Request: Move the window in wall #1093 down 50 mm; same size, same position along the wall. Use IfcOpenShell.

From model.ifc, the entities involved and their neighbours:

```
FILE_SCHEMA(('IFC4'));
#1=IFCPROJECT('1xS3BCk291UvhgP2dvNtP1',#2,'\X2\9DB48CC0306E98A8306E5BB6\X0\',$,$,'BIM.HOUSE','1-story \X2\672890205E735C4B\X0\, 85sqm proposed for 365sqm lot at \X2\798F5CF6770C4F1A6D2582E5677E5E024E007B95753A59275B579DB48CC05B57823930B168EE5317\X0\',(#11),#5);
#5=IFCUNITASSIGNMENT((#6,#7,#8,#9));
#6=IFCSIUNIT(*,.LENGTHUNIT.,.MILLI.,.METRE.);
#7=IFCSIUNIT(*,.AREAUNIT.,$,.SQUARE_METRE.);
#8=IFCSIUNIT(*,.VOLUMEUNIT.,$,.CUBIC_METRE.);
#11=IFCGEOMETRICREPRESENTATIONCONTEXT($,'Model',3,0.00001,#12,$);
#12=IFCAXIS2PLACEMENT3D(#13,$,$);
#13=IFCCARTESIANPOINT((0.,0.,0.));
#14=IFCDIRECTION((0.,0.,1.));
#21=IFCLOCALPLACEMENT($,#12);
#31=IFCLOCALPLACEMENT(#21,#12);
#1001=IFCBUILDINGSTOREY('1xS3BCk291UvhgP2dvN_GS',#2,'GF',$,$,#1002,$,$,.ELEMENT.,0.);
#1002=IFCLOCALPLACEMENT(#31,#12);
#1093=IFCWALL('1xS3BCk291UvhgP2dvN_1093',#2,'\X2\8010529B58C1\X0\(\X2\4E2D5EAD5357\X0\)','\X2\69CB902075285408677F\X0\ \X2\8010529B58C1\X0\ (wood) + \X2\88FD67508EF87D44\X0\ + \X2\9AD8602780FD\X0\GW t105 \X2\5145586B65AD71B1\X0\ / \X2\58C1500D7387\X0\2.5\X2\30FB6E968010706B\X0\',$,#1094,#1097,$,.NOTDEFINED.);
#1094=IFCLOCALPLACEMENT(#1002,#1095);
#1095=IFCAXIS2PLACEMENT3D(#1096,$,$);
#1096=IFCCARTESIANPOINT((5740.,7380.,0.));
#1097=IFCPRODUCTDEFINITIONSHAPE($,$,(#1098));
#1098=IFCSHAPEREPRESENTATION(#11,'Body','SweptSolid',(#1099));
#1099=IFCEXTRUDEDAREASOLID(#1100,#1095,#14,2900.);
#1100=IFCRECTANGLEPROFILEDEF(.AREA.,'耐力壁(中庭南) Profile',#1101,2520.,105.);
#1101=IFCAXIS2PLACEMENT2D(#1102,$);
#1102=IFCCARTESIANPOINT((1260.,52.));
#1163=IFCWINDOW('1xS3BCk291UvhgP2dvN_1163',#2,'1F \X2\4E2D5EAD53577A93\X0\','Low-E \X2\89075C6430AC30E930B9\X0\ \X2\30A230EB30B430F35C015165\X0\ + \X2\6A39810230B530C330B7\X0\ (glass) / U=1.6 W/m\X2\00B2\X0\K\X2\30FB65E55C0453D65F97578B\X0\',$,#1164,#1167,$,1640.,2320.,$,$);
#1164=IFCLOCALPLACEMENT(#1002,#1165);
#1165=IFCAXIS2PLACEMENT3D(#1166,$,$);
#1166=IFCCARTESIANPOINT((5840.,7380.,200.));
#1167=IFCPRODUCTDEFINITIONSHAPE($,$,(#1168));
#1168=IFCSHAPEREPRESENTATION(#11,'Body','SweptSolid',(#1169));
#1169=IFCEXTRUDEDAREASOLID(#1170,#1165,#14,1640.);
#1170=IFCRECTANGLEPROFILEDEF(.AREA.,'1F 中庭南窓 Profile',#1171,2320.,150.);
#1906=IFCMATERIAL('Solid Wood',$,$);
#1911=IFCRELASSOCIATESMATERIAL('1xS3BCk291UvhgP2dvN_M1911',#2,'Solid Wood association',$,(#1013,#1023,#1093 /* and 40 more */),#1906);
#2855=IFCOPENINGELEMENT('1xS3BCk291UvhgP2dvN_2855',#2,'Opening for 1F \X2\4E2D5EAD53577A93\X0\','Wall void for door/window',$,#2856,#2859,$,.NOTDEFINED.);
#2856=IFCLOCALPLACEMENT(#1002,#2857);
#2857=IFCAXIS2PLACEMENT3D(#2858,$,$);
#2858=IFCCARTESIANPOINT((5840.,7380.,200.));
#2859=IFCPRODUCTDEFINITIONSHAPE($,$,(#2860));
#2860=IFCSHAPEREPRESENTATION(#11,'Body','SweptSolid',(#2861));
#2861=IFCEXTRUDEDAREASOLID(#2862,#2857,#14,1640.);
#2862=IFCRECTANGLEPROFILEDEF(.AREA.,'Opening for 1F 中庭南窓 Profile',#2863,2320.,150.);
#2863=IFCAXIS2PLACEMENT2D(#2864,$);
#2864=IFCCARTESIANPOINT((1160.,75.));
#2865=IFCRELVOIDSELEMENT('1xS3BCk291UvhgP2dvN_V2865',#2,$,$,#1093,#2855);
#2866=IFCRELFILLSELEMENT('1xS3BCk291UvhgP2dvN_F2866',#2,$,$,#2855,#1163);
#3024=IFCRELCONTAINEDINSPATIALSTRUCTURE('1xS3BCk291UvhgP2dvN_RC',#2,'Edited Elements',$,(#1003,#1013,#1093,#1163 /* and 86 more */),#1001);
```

```python
import numpy as np
import ifcopenshell
import ifcopenshell.api.geometry
import ifcopenshell.util.placement
import ifcopenshell.util.unit

model = ifcopenshell.open("model.ifc")
unit_scale = ifcopenshell.util.unit.calculate_unit_scale(model)

window = model.by_guid("1xS3BCk291UvhgP2dvN_1163")
opening = window.FillsVoids[0].RelatingOpeningElement
dz = -0.05 / unit_scale

shift = np.array([0.0, 0.0, dz])
# The window is not placed relative to its opening, so move both.
for product in (opening, window):
    matrix = ifcopenshell.util.placement.get_local_placement(product.ObjectPlacement)
    matrix[:3, 3] += shift
    ifcopenshell.api.geometry.edit_object_placement(model, product=product, matrix=matrix, is_si=False)

print(f"moved by {dz * unit_scale:+.3f} m")

model.write("model-out.ifc")
```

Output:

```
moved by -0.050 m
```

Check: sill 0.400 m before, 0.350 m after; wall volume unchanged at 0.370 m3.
